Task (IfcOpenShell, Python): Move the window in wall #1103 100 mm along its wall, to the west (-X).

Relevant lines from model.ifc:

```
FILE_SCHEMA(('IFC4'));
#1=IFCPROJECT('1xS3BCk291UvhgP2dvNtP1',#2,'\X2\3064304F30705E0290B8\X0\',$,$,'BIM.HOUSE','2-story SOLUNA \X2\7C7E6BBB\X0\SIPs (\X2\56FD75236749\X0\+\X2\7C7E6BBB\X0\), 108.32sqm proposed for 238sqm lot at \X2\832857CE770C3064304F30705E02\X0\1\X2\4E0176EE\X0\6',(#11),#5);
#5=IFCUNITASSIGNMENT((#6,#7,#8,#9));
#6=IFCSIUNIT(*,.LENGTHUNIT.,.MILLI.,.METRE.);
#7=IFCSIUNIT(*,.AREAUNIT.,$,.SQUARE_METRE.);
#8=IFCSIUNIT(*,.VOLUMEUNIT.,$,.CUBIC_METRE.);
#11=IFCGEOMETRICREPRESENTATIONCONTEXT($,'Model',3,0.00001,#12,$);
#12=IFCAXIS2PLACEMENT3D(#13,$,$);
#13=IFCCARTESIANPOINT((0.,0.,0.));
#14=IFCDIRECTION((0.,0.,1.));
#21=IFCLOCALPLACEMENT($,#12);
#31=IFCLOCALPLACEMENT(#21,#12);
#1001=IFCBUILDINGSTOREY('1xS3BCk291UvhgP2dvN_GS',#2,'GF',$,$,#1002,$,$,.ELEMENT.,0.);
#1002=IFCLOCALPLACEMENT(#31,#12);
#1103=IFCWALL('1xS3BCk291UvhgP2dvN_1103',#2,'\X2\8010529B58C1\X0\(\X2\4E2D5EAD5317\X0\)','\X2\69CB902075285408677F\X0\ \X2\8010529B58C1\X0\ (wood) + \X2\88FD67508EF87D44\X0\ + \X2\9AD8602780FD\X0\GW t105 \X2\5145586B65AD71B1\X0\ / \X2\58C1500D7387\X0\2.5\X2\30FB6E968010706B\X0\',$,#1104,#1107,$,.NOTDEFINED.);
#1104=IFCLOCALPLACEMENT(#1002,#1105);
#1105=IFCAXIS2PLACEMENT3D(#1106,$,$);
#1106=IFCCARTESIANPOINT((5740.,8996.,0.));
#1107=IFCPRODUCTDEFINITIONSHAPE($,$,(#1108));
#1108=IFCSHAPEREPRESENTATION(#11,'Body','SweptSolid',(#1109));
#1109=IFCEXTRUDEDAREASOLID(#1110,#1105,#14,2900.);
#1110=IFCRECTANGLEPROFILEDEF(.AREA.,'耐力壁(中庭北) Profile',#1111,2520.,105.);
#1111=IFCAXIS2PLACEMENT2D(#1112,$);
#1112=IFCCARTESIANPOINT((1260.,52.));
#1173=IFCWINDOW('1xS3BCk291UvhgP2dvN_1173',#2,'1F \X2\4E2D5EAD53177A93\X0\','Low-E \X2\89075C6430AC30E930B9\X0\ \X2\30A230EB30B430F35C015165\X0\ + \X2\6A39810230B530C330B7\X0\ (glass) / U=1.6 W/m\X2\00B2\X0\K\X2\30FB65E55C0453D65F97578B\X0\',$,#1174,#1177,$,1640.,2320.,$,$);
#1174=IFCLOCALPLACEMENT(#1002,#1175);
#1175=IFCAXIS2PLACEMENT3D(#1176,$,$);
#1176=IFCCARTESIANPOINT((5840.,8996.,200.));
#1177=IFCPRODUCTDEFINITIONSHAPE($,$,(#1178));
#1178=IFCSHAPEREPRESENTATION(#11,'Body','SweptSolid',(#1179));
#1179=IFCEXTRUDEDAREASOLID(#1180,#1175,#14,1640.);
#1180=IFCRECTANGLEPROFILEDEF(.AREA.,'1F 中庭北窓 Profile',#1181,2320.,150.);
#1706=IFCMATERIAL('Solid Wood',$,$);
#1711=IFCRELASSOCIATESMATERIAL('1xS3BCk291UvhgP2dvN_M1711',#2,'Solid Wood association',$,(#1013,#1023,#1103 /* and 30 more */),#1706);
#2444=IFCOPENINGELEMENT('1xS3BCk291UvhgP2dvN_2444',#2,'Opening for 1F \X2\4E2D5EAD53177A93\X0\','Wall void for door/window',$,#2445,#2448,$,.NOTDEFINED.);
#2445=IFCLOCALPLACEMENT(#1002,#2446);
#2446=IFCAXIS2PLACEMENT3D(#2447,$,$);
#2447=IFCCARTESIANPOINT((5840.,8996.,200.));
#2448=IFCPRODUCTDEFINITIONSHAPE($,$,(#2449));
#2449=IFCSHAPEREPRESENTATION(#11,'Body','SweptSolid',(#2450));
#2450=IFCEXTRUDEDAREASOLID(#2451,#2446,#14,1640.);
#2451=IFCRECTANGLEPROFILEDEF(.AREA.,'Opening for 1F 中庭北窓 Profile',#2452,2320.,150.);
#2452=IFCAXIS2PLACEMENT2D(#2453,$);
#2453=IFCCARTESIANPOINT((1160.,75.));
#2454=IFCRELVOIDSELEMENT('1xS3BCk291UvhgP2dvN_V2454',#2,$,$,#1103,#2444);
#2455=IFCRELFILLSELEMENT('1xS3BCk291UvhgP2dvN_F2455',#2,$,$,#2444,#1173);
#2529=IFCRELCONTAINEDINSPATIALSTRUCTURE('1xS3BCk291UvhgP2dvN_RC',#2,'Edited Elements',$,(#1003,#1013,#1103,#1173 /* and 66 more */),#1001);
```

```python
import ifcopenshell
import ifcopenshell.api.geometry
import ifcopenshell.util.placement

model = ifcopenshell.open("model.ifc")

window = model.by_guid("1xS3BCk291UvhgP2dvN_1173")
opening = window.FillsVoids[0].RelatingOpeningElement
wall = opening.VoidsElements[0].RelatingBuildingElement

wall_matrix = ifcopenshell.util.placement.get_local_placement(wall.ObjectPlacement)
shift = wall_matrix[:3, 0] * -100.0
before = ifcopenshell.util.placement.get_local_placement(window.ObjectPlacement)[:3, 3].copy()

# The window is not placed relative to its opening, so move both.
for product in (opening, window):
    matrix = ifcopenshell.util.placement.get_local_placement(product.ObjectPlacement)
    matrix[:3, 3] += shift
    ifcopenshell.api.geometry.edit_object_placement(model, product=product, matrix=matrix, is_si=False)

after = ifcopenshell.util.placement.get_local_placement(window.ObjectPlacement)[:3, 3]
print("window moved by", (after - before).round(3) + 0.0)

model.write("model_edited.ifc")
```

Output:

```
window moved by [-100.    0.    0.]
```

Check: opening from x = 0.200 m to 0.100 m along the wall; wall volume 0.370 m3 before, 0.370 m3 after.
